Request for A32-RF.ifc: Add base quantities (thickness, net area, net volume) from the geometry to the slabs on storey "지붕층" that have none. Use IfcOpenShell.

First a look at what the model holds.

```python
import ifcopenshell
import ifcopenshell.util.element
import ifcopenshell.util.unit

model = ifcopenshell.open("A32-RF.ifc")
print(model.schema)
for unit_type in ("LENGTHUNIT", "AREAUNIT", "VOLUMEUNIT"):
    print(unit_type, ifcopenshell.util.unit.calculate_unit_scale(model, unit_type))
storey = next(s for s in model.by_type("IfcBuildingStorey") if s.Name == "지붕층")
slabs = [e for e in ifcopenshell.util.element.get_decomposition(storey) if e.is_a("IfcSlab")]
for e in sorted(slabs, key=lambda e: e.id()):
    print(e.id(), e.is_a(), e.Name, list(ifcopenshell.util.element.get_psets(e, qtos_only=True)), sep=" | ")
```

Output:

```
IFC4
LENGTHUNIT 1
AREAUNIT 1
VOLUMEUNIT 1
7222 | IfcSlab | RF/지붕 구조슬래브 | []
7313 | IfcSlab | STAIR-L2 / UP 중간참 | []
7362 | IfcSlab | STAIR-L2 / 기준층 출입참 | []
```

```python
import ifcopenshell
import ifcopenshell.api.pset
import ifcopenshell.geom
import ifcopenshell.util.element
import ifcopenshell.util.shape
import ifcopenshell.util.unit

model = ifcopenshell.open("A32-RF.ifc")
unit_scale = ifcopenshell.util.unit.calculate_unit_scale(model)
area_scale = ifcopenshell.util.unit.calculate_unit_scale(model, "AREAUNIT")
volume_scale = ifcopenshell.util.unit.calculate_unit_scale(model, "VOLUMEUNIT")
settings = ifcopenshell.geom.settings()

storey = next(s for s in model.by_type("IfcBuildingStorey") if s.Name == "지붕층")
slabs = [e for e in ifcopenshell.util.element.get_decomposition(storey) if e.is_a("IfcSlab")]

for e in sorted(slabs, key=lambda e: e.id()):
    if ifcopenshell.util.element.get_psets(e, qtos_only=True, should_inherit=False):
        continue
    # Geometry comes back in metres, in the element's own axes.
    shape = ifcopenshell.geom.create_shape(settings, e)
    values = {
        "Width": ifcopenshell.util.shape.get_z(shape.geometry) / unit_scale,
        "NetArea": ifcopenshell.util.shape.get_footprint_area(shape.geometry) / area_scale,
        "NetVolume": ifcopenshell.util.shape.get_volume(shape.geometry) / volume_scale,
    }
    qto = ifcopenshell.api.pset.add_qto(model, product=e, name="Qto_SlabBaseQuantities")
    ifcopenshell.api.pset.edit_qto(model, qto=qto, properties=values)
    print(e.id(), {k: round(v, 3) for k, v in values.items()})

model.write("A32-RF_rev.ifc")
```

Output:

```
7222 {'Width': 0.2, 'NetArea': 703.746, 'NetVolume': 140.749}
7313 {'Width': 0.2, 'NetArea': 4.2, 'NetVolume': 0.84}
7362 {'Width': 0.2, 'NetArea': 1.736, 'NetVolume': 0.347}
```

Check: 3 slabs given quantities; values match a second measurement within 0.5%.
